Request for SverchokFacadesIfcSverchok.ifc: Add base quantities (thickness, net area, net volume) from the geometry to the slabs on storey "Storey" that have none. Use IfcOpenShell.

First a look at what the model holds.

```python
import ifcopenshell
import ifcopenshell.util.element
import ifcopenshell.util.unit

model = ifcopenshell.open("SverchokFacadesIfcSverchok.ifc")
print(model.schema)
for unit_type in ("LENGTHUNIT", "AREAUNIT", "VOLUMEUNIT"):
    print(unit_type, ifcopenshell.util.unit.calculate_unit_scale(model, unit_type))
storey = next(s for s in model.by_type("IfcBuildingStorey") if s.Name == "Storey")
slabs = [e for e in ifcopenshell.util.element.get_decomposition(storey) if e.is_a("IfcSlab")]
for e in sorted(slabs, key=lambda e: e.id()):
    print(e.id(), e.is_a(), e.Name, list(ifcopenshell.util.element.get_psets(e, qtos_only=True)), sep=" | ")
```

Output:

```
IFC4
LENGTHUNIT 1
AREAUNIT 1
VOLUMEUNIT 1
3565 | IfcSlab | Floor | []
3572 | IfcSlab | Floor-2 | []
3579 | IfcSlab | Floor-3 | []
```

```python
import ifcopenshell
import ifcopenshell.api.pset
import ifcopenshell.geom
import ifcopenshell.util.element
import ifcopenshell.util.shape
import ifcopenshell.util.unit

model = ifcopenshell.open("SverchokFacadesIfcSverchok.ifc")
unit_scale = ifcopenshell.util.unit.calculate_unit_scale(model)
area_scale = ifcopenshell.util.unit.calculate_unit_scale(model, "AREAUNIT")
volume_scale = ifcopenshell.util.unit.calculate_unit_scale(model, "VOLUMEUNIT")
settings = ifcopenshell.geom.settings()

storey = next(s for s in model.by_type("IfcBuildingStorey") if s.Name == "Storey")
slabs = [e for e in ifcopenshell.util.element.get_decomposition(storey) if e.is_a("IfcSlab")]

for e in sorted(slabs, key=lambda e: e.id()):
    if ifcopenshell.util.element.get_psets(e, qtos_only=True, should_inherit=False):
        continue
    # Geometry comes back in metres, in the element's own axes.
    shape = ifcopenshell.geom.create_shape(settings, e)
    values = {
        "Width": ifcopenshell.util.shape.get_z(shape.geometry) / unit_scale,
        "NetArea": ifcopenshell.util.shape.get_footprint_area(shape.geometry) / area_scale,
        "NetVolume": ifcopenshell.util.shape.get_volume(shape.geometry) / volume_scale,
    }
    qto = ifcopenshell.api.pset.add_qto(model, product=e, name="Qto_SlabBaseQuantities")
    ifcopenshell.api.pset.edit_qto(model, qto=qto, properties=values)
    print(e.id(), {k: round(v, 3) for k, v in values.items()})

model.write("SverchokFacadesIfcSverchok-out.ifc")
```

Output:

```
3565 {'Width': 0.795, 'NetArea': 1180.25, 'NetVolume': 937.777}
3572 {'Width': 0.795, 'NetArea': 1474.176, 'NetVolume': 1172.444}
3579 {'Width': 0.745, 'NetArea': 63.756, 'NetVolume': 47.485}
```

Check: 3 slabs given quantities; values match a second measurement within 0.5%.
